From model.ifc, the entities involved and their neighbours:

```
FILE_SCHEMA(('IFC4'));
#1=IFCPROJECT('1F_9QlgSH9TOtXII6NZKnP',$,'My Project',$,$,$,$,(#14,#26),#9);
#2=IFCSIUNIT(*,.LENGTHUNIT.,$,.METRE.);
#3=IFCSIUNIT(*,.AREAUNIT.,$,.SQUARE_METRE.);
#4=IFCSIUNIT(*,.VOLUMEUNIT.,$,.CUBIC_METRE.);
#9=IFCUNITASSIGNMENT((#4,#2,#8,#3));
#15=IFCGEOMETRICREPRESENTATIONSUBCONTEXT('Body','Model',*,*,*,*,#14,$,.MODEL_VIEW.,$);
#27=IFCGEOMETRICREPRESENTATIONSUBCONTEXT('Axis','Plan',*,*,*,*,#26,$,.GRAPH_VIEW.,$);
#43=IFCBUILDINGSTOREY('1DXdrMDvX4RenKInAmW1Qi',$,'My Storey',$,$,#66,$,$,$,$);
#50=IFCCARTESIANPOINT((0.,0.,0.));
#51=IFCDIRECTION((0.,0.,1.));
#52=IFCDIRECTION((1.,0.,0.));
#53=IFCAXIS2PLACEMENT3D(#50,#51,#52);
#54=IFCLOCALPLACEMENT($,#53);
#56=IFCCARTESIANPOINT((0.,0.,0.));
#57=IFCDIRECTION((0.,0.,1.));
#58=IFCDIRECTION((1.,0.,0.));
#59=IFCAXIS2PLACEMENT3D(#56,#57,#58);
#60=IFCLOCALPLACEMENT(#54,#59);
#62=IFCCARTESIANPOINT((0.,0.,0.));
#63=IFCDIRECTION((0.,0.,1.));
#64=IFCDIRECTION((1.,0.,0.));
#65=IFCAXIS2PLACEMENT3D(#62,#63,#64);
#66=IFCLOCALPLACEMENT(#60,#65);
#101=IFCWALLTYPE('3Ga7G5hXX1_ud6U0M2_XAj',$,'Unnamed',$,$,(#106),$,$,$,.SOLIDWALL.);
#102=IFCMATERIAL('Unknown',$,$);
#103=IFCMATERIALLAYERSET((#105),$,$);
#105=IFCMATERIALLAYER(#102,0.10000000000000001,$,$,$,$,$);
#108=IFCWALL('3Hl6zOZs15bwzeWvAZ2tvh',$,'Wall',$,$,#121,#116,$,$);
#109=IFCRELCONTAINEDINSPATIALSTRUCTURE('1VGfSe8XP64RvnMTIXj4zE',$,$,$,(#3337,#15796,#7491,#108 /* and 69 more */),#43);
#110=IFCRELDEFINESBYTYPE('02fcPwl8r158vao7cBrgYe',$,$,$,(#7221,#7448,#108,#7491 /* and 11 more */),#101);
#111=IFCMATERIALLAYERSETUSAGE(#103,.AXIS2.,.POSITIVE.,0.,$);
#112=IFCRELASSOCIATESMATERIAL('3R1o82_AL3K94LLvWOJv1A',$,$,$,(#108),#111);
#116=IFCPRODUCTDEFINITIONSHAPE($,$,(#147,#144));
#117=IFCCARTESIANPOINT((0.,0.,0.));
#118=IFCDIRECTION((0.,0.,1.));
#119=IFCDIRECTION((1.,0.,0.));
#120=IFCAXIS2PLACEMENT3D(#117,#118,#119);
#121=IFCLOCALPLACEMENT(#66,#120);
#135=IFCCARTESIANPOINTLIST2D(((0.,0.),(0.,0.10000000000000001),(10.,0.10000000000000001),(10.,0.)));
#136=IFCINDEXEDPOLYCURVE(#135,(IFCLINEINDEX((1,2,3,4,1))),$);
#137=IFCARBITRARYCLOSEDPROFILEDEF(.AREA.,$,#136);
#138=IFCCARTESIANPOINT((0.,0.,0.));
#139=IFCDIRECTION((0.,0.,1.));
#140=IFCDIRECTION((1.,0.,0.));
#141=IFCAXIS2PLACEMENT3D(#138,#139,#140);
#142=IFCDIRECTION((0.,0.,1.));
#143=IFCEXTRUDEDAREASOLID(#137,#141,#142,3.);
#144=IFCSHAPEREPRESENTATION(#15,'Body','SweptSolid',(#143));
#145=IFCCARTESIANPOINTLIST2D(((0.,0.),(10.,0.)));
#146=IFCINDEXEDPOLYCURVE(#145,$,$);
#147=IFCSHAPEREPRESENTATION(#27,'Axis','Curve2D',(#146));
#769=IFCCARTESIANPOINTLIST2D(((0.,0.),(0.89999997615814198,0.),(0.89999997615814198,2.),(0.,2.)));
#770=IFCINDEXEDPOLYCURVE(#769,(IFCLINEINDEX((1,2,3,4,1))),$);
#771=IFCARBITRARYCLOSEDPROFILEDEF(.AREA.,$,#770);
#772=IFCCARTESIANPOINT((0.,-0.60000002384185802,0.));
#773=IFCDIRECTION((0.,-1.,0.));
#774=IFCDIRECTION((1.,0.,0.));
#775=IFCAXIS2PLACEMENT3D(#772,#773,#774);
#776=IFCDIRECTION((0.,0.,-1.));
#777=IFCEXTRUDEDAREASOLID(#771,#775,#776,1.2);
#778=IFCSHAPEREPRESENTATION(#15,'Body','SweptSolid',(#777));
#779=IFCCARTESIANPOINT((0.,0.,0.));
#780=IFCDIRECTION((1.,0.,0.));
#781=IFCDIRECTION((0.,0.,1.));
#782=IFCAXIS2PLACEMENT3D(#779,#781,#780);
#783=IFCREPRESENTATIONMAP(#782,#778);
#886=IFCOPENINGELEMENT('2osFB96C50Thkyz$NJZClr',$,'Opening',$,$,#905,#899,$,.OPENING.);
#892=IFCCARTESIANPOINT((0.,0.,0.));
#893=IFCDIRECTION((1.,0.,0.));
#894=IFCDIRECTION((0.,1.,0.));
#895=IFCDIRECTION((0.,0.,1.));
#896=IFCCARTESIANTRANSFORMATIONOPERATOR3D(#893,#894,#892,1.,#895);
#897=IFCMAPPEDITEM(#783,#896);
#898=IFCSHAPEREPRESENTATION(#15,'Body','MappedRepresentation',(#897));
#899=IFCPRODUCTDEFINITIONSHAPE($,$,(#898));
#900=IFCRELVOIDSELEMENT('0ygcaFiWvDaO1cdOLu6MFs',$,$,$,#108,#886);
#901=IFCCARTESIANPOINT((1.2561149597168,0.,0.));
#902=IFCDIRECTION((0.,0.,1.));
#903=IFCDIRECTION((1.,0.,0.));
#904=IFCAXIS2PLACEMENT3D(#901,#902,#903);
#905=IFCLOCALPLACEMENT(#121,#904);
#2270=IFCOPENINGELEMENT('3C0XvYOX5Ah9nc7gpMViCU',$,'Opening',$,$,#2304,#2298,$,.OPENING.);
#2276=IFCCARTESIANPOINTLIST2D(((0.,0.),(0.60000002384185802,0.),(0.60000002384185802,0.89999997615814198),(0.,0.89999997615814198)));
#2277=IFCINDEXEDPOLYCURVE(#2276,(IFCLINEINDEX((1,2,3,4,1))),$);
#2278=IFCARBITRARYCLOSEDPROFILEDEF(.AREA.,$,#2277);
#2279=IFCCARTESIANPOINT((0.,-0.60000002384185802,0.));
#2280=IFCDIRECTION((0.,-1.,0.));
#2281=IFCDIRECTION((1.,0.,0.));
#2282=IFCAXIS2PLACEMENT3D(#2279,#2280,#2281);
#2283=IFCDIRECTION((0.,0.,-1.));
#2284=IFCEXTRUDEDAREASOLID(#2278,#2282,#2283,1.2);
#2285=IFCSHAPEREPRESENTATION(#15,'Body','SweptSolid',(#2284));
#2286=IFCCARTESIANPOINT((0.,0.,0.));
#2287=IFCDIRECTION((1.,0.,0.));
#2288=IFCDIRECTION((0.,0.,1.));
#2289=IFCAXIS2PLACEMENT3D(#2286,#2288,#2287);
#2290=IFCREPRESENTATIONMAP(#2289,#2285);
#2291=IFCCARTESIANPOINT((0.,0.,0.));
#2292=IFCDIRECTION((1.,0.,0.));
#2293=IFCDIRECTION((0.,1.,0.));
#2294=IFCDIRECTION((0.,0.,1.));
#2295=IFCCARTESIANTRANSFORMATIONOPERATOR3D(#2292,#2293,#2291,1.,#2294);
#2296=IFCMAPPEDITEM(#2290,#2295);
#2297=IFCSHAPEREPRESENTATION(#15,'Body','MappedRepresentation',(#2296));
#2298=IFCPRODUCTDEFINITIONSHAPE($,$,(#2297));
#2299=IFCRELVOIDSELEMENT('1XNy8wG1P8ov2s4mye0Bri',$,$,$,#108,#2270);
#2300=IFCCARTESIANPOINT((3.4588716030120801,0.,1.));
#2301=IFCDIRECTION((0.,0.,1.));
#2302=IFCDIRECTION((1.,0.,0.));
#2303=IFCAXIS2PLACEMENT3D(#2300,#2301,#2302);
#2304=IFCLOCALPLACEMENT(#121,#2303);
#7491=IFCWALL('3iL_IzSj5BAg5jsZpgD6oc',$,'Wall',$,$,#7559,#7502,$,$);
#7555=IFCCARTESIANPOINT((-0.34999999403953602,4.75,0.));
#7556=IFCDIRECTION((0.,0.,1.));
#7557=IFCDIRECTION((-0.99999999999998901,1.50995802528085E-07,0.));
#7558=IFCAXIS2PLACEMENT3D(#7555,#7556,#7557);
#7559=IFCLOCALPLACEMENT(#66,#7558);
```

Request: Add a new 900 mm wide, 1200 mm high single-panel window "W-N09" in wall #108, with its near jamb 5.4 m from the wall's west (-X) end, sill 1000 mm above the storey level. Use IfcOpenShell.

```python
import numpy as np
import ifcopenshell
import ifcopenshell.api.feature
import ifcopenshell.api.geometry
import ifcopenshell.api.root
import ifcopenshell.api.spatial
import ifcopenshell.geom
import ifcopenshell.util.element
import ifcopenshell.util.placement
import ifcopenshell.util.representation
import ifcopenshell.util.shape
import ifcopenshell.util.unit

model = ifcopenshell.open("model.ifc")
unit_scale = ifcopenshell.util.unit.calculate_unit_scale(model)
settings = ifcopenshell.geom.settings()


def volume(element):
    """Net volume in cubic metres, openings subtracted."""
    shape = ifcopenshell.geom.create_shape(settings, element)
    return ifcopenshell.util.shape.get_volume(shape.geometry)


wall = model.by_guid("3Hl6zOZs15bwzeWvAZ2tvh")
storey = ifcopenshell.util.element.get_container(wall, ifc_class="IfcBuildingStorey")
context = ifcopenshell.util.representation.get_context(model, "Model", "Body", "MODEL_VIEW")
before = volume(wall)

width, height, from_end, sill = 0.9, 1.2, 5.4, 1  # metres

# The wall runs along its own X axis, and the end named is its -X end.
wall_shape = ifcopenshell.geom.create_shape(settings, wall)
x, y, z = ifcopenshell.util.shape.get_vertices(wall_shape.geometry).T
start = x.min() + from_end
face, thickness = float(y.min()), float(y.max() - y.min())
wall_matrix = ifcopenshell.util.placement.get_local_placement(wall.ObjectPlacement)
level = ifcopenshell.util.placement.get_local_placement(storey.ObjectPlacement)[2, 3]


def in_wall(x, y):
    """Placement at x, y metres in the wall's axes, at sill height."""
    matrix = wall_matrix.copy()
    matrix[:, 3] = wall_matrix @ np.array([x / unit_scale, y / unit_scale, 0.0, 1.0])
    matrix[2, 3] = level + sill / unit_scale
    return matrix


# Opening: a box that overshoots both wall faces by 50 mm.
opening = ifcopenshell.api.root.create_entity(model, ifc_class="IfcOpeningElement", predefined_type="OPENING")
box = ifcopenshell.api.geometry.add_wall_representation(
    model, context=context, length=width, height=height, thickness=thickness + 0.1
)
ifcopenshell.api.geometry.assign_representation(model, product=opening, representation=box)
ifcopenshell.api.geometry.edit_object_placement(model, product=opening, matrix=in_wall(start, face - 0.05), is_si=False)
ifcopenshell.api.feature.add_feature(model, feature=opening, element=wall)

window = ifcopenshell.api.root.create_entity(model, ifc_class="IfcWindow", name="W-N09", predefined_type="WINDOW")
window.OverallWidth, window.OverallHeight = width / unit_scale, height / unit_scale
window.PartitioningType = "SINGLE_PANEL"
body = ifcopenshell.api.geometry.add_window_representation(
    model,
    context=context,
    overall_width=window.OverallWidth,
    overall_height=window.OverallHeight,
    partition_type="SINGLE_PANEL",
)
ifcopenshell.api.geometry.assign_representation(model, product=window, representation=body)
ifcopenshell.api.spatial.assign_container(model, products=[window], relating_structure=storey)
ifcopenshell.api.feature.add_filling(model, opening=opening, element=window)

# Centre the window in the wall's thickness.
ifcopenshell.api.geometry.edit_object_placement(model, product=window, matrix=in_wall(start, face), is_si=False)
window_shape = ifcopenshell.geom.create_shape(settings, window)
depth = ifcopenshell.util.shape.get_vertices(window_shape.geometry)[:, 1]
offset = face + thickness / 2 - (depth.min() + depth.max()) / 2
ifcopenshell.api.geometry.edit_object_placement(model, product=window, matrix=in_wall(start, offset), is_si=False)

after = volume(wall)

print(f"wall volume {before:.3f} -> {after:.3f} m3")

model.write("model_edited.ifc")
```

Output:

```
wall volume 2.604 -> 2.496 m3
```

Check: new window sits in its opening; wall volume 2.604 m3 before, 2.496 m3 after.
